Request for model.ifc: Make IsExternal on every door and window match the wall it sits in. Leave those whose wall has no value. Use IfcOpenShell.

First a look at what the model holds.

```python
import ifcopenshell
import ifcopenshell.util.element

model = ifcopenshell.open("model.ifc")
print(model.schema)
seen = {}
for e in model.by_type("IfcDoor") + model.by_type("IfcWindow"):
    if not e.FillsVoids:
        continue
    host = e.FillsVoids[0].RelatingOpeningElement.VoidsElements[0].RelatingBuildingElement
    own = ifcopenshell.util.element.get_pset(e, f"Pset_{e.is_a()[3:].removesuffix('StandardCase')}Common", "IsExternal")
    wall = ifcopenshell.util.element.get_pset(host, "Pset_WallCommon", "IsExternal")
    seen[e.is_a(), own, wall] = seen.get((e.is_a(), own, wall), 0) + 1
for (cls, own, wall), count in sorted(seen.items(), key=str):
    print(count, cls, "IsExternal:", own, "| host wall:", wall)
```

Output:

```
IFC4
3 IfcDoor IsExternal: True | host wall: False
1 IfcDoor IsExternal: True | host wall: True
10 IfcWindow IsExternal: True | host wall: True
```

```python
import ifcopenshell
import ifcopenshell.api.pset
import ifcopenshell.util.element

model = ifcopenshell.open("model.ifc")

count = 0
for ifc_class, pset_name in (("IfcDoor", "Pset_DoorCommon"), ("IfcWindow", "Pset_WindowCommon")):
    for e in model.by_type(ifc_class):
        if not e.FillsVoids:
            continue
        host = e.FillsVoids[0].RelatingOpeningElement.VoidsElements[0].RelatingBuildingElement
        external = ifcopenshell.util.element.get_pset(host, "Pset_WallCommon", "IsExternal")
        if external is None or ifcopenshell.util.element.get_pset(e, pset_name, "IsExternal") == external:
            continue
        pset = ifcopenshell.api.pset.add_pset(model, product=e, name=pset_name)
        ifcopenshell.api.pset.edit_pset(model, pset=pset, properties={"IsExternal": external})
        count += 1

print(count, "updated")

model.write("model-out.ifc")
```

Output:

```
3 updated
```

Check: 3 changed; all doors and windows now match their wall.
